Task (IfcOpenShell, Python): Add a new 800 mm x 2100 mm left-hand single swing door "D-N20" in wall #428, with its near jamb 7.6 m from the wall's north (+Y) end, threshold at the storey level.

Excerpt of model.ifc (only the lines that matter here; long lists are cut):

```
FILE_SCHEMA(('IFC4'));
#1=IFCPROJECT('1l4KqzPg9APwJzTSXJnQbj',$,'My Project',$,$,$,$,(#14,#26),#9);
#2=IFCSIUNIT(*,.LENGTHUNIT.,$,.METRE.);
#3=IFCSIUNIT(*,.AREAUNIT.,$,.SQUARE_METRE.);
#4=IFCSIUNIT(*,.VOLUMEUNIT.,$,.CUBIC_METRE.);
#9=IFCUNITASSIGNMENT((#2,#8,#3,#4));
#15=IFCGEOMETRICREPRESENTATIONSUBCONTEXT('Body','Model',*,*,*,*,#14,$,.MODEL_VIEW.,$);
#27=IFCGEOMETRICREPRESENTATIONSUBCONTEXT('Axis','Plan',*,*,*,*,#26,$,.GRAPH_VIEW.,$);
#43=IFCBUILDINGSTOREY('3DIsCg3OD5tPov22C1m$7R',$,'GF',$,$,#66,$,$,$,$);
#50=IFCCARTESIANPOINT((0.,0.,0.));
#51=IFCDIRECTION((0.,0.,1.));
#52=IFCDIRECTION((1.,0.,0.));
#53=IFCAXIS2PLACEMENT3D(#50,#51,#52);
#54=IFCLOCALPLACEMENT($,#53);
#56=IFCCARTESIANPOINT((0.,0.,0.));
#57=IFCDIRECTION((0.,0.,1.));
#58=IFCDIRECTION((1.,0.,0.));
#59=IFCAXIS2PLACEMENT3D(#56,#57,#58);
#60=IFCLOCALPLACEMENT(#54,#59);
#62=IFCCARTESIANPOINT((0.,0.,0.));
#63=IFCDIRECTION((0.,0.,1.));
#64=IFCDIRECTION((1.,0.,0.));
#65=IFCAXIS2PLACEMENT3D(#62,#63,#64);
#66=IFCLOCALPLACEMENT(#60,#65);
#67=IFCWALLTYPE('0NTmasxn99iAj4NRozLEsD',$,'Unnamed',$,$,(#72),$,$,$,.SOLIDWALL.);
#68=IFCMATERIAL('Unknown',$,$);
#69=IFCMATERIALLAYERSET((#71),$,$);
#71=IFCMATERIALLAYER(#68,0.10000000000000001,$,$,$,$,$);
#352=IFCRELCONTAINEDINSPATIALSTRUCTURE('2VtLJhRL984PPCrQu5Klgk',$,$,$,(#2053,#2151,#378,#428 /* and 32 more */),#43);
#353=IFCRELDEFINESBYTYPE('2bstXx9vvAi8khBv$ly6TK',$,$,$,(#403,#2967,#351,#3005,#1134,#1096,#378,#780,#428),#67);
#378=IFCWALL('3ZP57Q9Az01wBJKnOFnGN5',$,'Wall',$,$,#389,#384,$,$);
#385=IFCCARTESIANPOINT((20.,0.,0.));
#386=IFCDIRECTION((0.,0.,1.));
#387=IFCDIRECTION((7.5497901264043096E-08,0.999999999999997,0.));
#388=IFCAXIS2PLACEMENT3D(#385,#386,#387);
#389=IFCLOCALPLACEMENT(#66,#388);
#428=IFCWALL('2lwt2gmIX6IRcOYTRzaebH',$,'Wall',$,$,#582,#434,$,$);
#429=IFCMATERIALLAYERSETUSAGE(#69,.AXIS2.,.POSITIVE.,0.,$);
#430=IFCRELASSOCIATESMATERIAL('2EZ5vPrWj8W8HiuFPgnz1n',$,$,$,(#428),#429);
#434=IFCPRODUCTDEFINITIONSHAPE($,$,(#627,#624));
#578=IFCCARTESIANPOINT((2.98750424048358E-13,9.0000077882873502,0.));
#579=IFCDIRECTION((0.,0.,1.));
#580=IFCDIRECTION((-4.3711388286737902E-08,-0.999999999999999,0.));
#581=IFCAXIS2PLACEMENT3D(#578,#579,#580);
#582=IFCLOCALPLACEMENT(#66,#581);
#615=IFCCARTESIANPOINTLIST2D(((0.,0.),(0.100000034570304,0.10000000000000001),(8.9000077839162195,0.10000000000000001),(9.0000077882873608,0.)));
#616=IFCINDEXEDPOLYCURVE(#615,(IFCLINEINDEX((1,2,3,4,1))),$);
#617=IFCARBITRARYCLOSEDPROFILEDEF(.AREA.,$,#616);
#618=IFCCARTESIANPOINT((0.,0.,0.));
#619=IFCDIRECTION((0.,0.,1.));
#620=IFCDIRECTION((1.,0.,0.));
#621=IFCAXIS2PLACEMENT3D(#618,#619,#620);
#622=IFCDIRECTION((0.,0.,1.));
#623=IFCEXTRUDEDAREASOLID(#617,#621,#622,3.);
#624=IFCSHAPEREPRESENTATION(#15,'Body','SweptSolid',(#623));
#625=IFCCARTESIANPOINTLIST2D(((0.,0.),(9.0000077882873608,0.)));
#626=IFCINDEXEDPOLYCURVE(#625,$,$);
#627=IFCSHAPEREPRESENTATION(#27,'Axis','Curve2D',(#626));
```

```python
import numpy as np
import ifcopenshell
import ifcopenshell.api.feature
import ifcopenshell.api.geometry
import ifcopenshell.api.root
import ifcopenshell.api.spatial
import ifcopenshell.geom
import ifcopenshell.util.element
import ifcopenshell.util.placement
import ifcopenshell.util.representation
import ifcopenshell.util.shape
import ifcopenshell.util.unit

model = ifcopenshell.open("model.ifc")
unit_scale = ifcopenshell.util.unit.calculate_unit_scale(model)
settings = ifcopenshell.geom.settings()


def volume(element):
    """Net volume in cubic metres, openings subtracted."""
    shape = ifcopenshell.geom.create_shape(settings, element)
    return ifcopenshell.util.shape.get_volume(shape.geometry)


wall = model.by_guid("2lwt2gmIX6IRcOYTRzaebH")
storey = ifcopenshell.util.element.get_container(wall, ifc_class="IfcBuildingStorey")
context = ifcopenshell.util.representation.get_context(model, "Model", "Body", "MODEL_VIEW")
before = volume(wall)

width, height, from_end, sill = 0.8, 2.1, 7.6, 0.0  # metres

# The wall runs along its own X axis, and the end named is its -X end.
wall_shape = ifcopenshell.geom.create_shape(settings, wall)
x, y, z = ifcopenshell.util.shape.get_vertices(wall_shape.geometry).T
start = x.min() + from_end
face, thickness = float(y.min()), float(y.max() - y.min())
wall_matrix = ifcopenshell.util.placement.get_local_placement(wall.ObjectPlacement)
level = ifcopenshell.util.placement.get_local_placement(storey.ObjectPlacement)[2, 3]


def in_wall(x, y):
    """Placement at x, y metres in the wall's axes, at sill height."""
    matrix = wall_matrix.copy()
    matrix[:, 3] = wall_matrix @ np.array([x / unit_scale, y / unit_scale, 0.0, 1.0])
    matrix[2, 3] = level + sill / unit_scale
    return matrix


# Opening: a box that overshoots both wall faces by 50 mm.
opening = ifcopenshell.api.root.create_entity(model, ifc_class="IfcOpeningElement", predefined_type="OPENING")
box = ifcopenshell.api.geometry.add_wall_representation(
    model, context=context, length=width, height=height, thickness=thickness + 0.1
)
ifcopenshell.api.geometry.assign_representation(model, product=opening, representation=box)
ifcopenshell.api.geometry.edit_object_placement(model, product=opening, matrix=in_wall(start, face - 0.05), is_si=False)
ifcopenshell.api.feature.add_feature(model, feature=opening, element=wall)

door = ifcopenshell.api.root.create_entity(model, ifc_class="IfcDoor", name="D-N20", predefined_type="DOOR")
door.OverallWidth, door.OverallHeight = width / unit_scale, height / unit_scale
door.OperationType = "SINGLE_SWING_LEFT"
body = ifcopenshell.api.geometry.add_door_representation(
    model,
    context=context,
    overall_width=door.OverallWidth,
    overall_height=door.OverallHeight,
    operation_type="SINGLE_SWING_LEFT",
    lining_properties={"LiningDepth": thickness / unit_scale, "ThresholdDepth": thickness / unit_scale},
)
ifcopenshell.api.geometry.assign_representation(model, product=door, representation=body)
ifcopenshell.api.spatial.assign_container(model, products=[door], relating_structure=storey)
ifcopenshell.api.feature.add_filling(model, opening=opening, element=door)

# The lining spans the wall, so the door starts at the wall face.
ifcopenshell.api.geometry.edit_object_placement(model, product=door, matrix=in_wall(start, face), is_si=False)

after = volume(wall)

print(f"wall volume {before:.3f} -> {after:.3f} m3")

model.write("model_edited.ifc")
```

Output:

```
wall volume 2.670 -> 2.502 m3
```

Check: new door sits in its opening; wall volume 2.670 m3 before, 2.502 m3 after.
